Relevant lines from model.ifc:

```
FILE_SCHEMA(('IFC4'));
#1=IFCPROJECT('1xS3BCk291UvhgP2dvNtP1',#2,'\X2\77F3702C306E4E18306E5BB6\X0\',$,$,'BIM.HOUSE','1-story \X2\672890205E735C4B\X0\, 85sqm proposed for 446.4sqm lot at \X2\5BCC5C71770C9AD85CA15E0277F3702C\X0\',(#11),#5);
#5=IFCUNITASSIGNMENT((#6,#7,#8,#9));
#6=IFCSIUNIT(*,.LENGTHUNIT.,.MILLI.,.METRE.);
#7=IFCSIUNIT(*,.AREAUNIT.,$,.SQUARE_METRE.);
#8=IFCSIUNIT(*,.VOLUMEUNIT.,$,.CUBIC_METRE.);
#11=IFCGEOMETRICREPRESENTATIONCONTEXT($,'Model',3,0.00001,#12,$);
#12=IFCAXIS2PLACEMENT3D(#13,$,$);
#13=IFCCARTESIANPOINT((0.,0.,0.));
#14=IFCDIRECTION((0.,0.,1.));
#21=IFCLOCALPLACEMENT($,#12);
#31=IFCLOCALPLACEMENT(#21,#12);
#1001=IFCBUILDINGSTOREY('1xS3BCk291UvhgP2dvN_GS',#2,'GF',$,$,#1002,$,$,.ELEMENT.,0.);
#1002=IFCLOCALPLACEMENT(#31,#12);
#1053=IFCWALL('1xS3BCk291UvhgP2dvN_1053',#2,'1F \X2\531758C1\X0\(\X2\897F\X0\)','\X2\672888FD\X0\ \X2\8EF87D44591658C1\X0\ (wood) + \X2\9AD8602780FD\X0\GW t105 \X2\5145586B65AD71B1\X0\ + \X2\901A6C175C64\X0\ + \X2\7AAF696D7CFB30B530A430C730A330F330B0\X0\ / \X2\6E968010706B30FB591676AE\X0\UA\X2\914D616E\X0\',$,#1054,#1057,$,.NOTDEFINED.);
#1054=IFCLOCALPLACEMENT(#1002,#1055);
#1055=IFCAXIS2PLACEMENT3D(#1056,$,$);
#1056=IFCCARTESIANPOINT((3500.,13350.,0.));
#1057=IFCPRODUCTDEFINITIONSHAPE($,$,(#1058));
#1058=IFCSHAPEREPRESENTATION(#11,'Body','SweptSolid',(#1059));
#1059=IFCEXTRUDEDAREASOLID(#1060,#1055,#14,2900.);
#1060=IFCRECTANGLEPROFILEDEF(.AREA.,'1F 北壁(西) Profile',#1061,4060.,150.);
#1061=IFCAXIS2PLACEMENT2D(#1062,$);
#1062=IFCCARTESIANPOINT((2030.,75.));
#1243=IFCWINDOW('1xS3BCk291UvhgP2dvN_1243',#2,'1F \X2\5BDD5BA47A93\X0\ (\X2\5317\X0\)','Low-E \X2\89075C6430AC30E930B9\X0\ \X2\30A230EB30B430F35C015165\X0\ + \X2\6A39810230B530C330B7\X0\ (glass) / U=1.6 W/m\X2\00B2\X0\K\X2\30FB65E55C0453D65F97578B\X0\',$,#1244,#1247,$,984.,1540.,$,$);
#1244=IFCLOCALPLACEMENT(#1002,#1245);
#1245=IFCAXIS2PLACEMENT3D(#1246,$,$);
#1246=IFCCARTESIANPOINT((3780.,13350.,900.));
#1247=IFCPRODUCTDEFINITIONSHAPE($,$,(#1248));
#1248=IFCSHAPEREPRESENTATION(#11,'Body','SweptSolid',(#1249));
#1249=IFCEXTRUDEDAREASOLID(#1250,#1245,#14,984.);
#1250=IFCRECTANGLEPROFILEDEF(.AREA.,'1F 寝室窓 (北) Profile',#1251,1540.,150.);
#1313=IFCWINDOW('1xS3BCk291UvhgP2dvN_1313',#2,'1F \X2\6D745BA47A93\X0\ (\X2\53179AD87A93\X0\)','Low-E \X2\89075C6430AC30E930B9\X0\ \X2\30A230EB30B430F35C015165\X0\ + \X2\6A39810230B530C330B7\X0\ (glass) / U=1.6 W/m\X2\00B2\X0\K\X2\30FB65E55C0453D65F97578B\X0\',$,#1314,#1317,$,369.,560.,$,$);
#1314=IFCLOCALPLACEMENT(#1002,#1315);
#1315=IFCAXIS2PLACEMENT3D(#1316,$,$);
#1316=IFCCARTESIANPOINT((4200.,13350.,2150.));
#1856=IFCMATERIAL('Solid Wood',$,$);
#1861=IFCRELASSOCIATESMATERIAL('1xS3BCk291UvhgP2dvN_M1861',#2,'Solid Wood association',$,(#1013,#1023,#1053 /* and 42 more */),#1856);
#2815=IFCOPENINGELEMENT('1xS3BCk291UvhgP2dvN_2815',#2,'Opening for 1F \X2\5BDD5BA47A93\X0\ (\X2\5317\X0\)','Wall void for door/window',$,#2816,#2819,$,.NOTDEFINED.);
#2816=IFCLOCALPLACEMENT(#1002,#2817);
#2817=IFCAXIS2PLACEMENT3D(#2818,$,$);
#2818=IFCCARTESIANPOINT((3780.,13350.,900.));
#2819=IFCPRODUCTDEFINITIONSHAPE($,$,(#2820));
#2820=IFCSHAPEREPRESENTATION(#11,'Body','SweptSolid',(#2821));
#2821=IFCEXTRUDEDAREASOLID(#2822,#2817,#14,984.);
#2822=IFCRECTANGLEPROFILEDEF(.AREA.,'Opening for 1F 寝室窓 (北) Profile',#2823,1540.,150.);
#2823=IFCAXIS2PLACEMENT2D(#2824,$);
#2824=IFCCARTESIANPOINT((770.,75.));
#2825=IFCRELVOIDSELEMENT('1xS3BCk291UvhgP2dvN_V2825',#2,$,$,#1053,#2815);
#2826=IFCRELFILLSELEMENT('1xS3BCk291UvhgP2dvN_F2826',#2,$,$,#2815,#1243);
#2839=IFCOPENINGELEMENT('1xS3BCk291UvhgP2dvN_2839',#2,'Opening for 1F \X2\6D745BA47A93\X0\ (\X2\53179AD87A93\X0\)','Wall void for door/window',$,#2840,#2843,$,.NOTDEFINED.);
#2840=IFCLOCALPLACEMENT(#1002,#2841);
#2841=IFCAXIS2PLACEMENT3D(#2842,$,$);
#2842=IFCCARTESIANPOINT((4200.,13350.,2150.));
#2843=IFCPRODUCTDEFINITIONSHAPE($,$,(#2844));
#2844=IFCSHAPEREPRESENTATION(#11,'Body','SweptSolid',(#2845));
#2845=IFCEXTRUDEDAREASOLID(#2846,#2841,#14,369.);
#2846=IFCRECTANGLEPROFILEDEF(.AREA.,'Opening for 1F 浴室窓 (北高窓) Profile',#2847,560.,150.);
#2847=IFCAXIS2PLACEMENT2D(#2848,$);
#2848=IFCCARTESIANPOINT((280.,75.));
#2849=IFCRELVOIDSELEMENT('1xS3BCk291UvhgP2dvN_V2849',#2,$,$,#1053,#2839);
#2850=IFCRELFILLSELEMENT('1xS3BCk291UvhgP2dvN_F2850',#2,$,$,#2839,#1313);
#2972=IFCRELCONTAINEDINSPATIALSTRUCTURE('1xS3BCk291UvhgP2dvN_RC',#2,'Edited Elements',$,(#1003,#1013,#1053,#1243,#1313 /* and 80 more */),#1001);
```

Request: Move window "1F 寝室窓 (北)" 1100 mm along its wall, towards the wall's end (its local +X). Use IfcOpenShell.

```python
import ifcopenshell
import ifcopenshell.api.geometry
import ifcopenshell.util.placement
import ifcopenshell.util.unit

model = ifcopenshell.open("model.ifc")
unit_scale = ifcopenshell.util.unit.calculate_unit_scale(model)

window = model.by_id(1243)
opening = window.FillsVoids[0].RelatingOpeningElement
wall = opening.VoidsElements[0].RelatingBuildingElement

wall_matrix = ifcopenshell.util.placement.get_local_placement(wall.ObjectPlacement)
shift = wall_matrix[:3, 0] * 1.1 / unit_scale
before = ifcopenshell.util.placement.get_local_placement(window.ObjectPlacement)[:3, 3].copy()

# The window is not placed relative to its opening, so move both.
for product in (opening, window):
    matrix = ifcopenshell.util.placement.get_local_placement(product.ObjectPlacement)
    matrix[:3, 3] += shift
    ifcopenshell.api.geometry.edit_object_placement(model, product=product, matrix=matrix, is_si=False)

after = ifcopenshell.util.placement.get_local_placement(window.ObjectPlacement)[:3, 3]
print("window moved by", (after - before).round(3) + 0.0)

model.write("model_updated.ifc")
```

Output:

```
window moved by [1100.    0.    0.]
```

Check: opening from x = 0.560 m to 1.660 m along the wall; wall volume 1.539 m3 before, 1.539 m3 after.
